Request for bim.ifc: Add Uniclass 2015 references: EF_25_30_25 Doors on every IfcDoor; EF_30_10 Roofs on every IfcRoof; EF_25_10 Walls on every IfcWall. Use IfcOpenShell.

First a look at what the model holds.

```python
import ifcopenshell

model = ifcopenshell.open("bim.ifc")
print(model.schema)
print("classifications:", [c.Name for c in model.by_type("IfcClassification")])
for ifc_class in ("IfcDoor", "IfcRoof", "IfcStair", "IfcWall", "IfcWindow"):
    print(ifc_class, len(model.by_type(ifc_class)))
```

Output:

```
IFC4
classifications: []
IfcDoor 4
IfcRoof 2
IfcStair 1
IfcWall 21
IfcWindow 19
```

```python
import ifcopenshell
import ifcopenshell.api.classification

model = ifcopenshell.open("bim.ifc")

system = ifcopenshell.api.classification.add_classification(model, classification="Uniclass 2015")

codes = {
    "IfcDoor": ("EF_25_30_25", "Doors"),
    "IfcRoof": ("EF_30_10", "Roofs"),
    "IfcWall": ("EF_25_10", "Walls"),
}
for ifc_class, (code, name) in codes.items():
    products = model.by_type(ifc_class)
    ifcopenshell.api.classification.add_reference(
        model, products=products, classification=system, identification=code, name=name
    )
    print(code, len(products))

model.write("bim_updated.ifc")
```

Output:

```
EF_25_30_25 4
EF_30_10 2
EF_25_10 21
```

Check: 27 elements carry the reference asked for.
